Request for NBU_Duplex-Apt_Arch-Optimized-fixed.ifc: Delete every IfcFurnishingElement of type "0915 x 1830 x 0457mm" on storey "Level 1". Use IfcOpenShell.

First a look at what the model holds.

```python
import ifcopenshell
import ifcopenshell.util.element

model = ifcopenshell.open("NBU_Duplex-Apt_Arch-Optimized-fixed.ifc")
print(model.schema)
storey = next(s for s in model.by_type("IfcBuildingStorey") if s.Name == "Level 1")
furniture = [e for e in ifcopenshell.util.element.get_decomposition(storey) if e.is_a("IfcFurnishingElement")]
seen = {}
for e in furniture:
    element_type = ifcopenshell.util.element.get_type(e)
    name = element_type.Name if element_type not in (None, e) else None
    seen[name] = seen.get(name, 0) + 1
for name, count in sorted(seen.items(), key=str):
    print(count, "x", name)
```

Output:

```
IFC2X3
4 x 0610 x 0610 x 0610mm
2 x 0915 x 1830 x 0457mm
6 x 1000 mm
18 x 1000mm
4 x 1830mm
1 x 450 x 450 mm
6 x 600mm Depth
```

```python
import ifcopenshell
import ifcopenshell.api.root
import ifcopenshell.util.element

model = ifcopenshell.open("NBU_Duplex-Apt_Arch-Optimized-fixed.ifc")

storey = next(s for s in model.by_type("IfcBuildingStorey") if s.Name == "Level 1")
furniture = [e for e in ifcopenshell.util.element.get_decomposition(storey) if e.is_a("IfcFurnishingElement")]
targets = [e for e in furniture if (t := ifcopenshell.util.element.get_type(e)) not in (None, e) and t.Name == "0915 x 1830 x 0457mm"]

for e in targets:
    ifcopenshell.api.root.remove_product(model, product=e)
print(len(targets), "removed")

model.write("NBU_Duplex-Apt_Arch-Optimized-fixed-out.ifc")
```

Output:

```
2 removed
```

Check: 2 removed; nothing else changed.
